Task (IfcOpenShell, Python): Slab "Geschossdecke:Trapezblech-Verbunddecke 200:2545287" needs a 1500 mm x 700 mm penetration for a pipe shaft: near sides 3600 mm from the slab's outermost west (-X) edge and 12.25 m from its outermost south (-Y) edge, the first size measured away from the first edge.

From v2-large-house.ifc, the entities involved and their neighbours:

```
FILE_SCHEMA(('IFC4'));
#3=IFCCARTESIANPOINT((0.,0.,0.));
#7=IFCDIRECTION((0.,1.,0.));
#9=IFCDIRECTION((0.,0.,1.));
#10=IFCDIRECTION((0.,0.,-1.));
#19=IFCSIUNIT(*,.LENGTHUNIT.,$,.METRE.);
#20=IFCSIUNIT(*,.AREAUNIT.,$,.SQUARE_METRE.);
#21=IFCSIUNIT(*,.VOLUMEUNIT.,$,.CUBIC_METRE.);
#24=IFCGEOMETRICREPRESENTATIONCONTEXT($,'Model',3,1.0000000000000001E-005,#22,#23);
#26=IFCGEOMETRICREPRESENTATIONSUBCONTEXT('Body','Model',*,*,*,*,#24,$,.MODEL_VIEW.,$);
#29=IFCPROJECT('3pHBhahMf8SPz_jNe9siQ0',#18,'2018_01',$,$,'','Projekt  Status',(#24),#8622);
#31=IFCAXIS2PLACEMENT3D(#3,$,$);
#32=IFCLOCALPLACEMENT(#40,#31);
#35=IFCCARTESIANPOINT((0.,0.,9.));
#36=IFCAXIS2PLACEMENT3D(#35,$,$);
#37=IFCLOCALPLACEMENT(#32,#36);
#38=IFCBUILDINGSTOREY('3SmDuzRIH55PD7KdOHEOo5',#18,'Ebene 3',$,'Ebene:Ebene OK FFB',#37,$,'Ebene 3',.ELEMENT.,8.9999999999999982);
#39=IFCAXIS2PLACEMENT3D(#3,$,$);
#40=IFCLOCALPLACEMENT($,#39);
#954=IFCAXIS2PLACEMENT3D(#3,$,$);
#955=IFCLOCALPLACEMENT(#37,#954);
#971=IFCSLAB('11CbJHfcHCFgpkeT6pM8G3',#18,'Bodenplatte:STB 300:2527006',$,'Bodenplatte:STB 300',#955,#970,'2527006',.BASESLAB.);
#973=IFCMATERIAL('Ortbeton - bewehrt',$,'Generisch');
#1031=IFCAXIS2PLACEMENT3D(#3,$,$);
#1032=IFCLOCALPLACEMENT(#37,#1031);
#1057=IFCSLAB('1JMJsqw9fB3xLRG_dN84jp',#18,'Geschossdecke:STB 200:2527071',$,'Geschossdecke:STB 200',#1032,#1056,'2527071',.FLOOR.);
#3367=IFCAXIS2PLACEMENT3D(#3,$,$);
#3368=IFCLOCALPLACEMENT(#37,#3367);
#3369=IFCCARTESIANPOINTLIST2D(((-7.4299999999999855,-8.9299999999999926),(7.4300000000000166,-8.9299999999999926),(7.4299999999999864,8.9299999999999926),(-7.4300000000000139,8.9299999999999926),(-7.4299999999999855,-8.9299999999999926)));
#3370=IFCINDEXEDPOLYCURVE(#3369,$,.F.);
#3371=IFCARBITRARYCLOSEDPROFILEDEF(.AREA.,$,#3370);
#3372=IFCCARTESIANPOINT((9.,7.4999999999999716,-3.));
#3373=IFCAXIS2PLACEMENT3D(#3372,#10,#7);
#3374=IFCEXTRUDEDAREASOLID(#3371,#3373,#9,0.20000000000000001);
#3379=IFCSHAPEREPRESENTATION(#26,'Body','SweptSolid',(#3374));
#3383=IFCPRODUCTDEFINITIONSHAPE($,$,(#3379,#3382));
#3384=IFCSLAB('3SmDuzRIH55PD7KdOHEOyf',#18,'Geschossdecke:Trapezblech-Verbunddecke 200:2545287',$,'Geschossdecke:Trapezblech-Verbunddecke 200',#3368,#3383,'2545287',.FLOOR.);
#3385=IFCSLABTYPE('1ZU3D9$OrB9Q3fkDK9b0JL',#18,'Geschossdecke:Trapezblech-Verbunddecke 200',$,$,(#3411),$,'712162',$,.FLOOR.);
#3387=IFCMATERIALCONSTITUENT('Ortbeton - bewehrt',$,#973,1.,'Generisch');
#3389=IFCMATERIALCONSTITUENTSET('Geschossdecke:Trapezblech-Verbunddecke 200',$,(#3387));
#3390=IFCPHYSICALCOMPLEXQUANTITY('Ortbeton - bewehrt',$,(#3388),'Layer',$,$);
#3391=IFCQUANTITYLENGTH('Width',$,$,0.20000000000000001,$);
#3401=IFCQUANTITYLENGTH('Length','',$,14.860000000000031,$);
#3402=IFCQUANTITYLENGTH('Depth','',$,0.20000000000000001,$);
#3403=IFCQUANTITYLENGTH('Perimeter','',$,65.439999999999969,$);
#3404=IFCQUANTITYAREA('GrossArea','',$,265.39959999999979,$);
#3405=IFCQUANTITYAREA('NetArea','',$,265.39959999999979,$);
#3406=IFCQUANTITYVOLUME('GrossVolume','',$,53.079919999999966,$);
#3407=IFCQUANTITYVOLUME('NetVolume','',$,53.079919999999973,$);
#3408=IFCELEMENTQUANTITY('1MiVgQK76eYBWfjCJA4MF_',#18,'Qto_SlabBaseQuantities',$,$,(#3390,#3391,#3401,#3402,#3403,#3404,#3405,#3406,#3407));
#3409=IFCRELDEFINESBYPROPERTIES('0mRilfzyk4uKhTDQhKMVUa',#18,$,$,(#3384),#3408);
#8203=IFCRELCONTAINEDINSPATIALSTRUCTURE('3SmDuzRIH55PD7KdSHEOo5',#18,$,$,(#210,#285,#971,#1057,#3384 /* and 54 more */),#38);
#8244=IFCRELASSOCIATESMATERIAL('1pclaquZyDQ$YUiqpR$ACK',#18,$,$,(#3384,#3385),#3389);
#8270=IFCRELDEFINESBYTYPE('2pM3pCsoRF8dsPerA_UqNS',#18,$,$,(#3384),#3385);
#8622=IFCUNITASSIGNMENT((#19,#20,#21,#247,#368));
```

```python
import numpy as np
import ifcopenshell
import ifcopenshell.api.feature
import ifcopenshell.api.geometry
import ifcopenshell.api.pset
import ifcopenshell.api.root
import ifcopenshell.geom
import ifcopenshell.util.element
import ifcopenshell.util.placement
import ifcopenshell.util.representation
import ifcopenshell.util.shape
import ifcopenshell.util.unit

model = ifcopenshell.open("v2-large-house.ifc")
unit_scale = ifcopenshell.util.unit.calculate_unit_scale(model)
area_scale = ifcopenshell.util.unit.calculate_unit_scale(model, "AREAUNIT")
volume_scale = ifcopenshell.util.unit.calculate_unit_scale(model, "VOLUMEUNIT")
settings = ifcopenshell.geom.settings()


def volume(element):
    """Net volume in cubic metres, openings subtracted."""
    shape = ifcopenshell.geom.create_shape(settings, element)
    return ifcopenshell.util.shape.get_volume(shape.geometry)


slab = model.by_guid("3SmDuzRIH55PD7KdOHEOyf")
before = volume(slab)

# Extent in the slab's own axes, in metres. The edges named are its -X and -Y sides.
slab_shape = ifcopenshell.geom.create_shape(settings, slab)
vertices = ifcopenshell.util.shape.get_vertices(slab_shape.geometry)
x_min, y_min, bottom = vertices.min(axis=0)
top = vertices[:, 2].max()

opening = ifcopenshell.api.root.create_entity(model, ifc_class="IfcOpeningElement", name="Pipe shaft opening", predefined_type="OPENING")
context = ifcopenshell.util.representation.get_context(model, "Model", "Body", "MODEL_VIEW")
width, depth = 1.5, 0.7
outline = [(0.0, 0.0), (width, 0.0), (width, depth), (0.0, depth), (0.0, 0.0)]
# Overshoot both faces by 50 mm so the cut is clean.
shape = ifcopenshell.api.geometry.add_slab_representation(
    model, context=context, depth=top - bottom + 0.1, polyline=outline
)
ifcopenshell.api.geometry.assign_representation(model, product=opening, representation=shape)

matrix = ifcopenshell.util.placement.get_local_placement(slab.ObjectPlacement)
matrix[:, 3] = matrix @ np.append(np.array([x_min + 3.6, y_min + 12.25, bottom - 0.05]) / unit_scale, 1.0)
ifcopenshell.api.geometry.edit_object_placement(model, product=opening, matrix=matrix, is_si=False)
ifcopenshell.api.feature.add_feature(model, feature=opening, element=slab)

after = volume(slab)

# Update the slab's stored quantities.
qto = model.by_id(ifcopenshell.util.element.get_pset(slab, "Qto_SlabBaseQuantities", should_inherit=False)["id"])
ifcopenshell.api.pset.edit_qto(model, qto=qto, properties={
    "NetArea": after / (top - bottom) / area_scale,
    "NetVolume": after / volume_scale,
})

print(f"slab volume {before:.3f} -> {after:.3f} m3")

model.write("v2-large-house_rev.ifc")
```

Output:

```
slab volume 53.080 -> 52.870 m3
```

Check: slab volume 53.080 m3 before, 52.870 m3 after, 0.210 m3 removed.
